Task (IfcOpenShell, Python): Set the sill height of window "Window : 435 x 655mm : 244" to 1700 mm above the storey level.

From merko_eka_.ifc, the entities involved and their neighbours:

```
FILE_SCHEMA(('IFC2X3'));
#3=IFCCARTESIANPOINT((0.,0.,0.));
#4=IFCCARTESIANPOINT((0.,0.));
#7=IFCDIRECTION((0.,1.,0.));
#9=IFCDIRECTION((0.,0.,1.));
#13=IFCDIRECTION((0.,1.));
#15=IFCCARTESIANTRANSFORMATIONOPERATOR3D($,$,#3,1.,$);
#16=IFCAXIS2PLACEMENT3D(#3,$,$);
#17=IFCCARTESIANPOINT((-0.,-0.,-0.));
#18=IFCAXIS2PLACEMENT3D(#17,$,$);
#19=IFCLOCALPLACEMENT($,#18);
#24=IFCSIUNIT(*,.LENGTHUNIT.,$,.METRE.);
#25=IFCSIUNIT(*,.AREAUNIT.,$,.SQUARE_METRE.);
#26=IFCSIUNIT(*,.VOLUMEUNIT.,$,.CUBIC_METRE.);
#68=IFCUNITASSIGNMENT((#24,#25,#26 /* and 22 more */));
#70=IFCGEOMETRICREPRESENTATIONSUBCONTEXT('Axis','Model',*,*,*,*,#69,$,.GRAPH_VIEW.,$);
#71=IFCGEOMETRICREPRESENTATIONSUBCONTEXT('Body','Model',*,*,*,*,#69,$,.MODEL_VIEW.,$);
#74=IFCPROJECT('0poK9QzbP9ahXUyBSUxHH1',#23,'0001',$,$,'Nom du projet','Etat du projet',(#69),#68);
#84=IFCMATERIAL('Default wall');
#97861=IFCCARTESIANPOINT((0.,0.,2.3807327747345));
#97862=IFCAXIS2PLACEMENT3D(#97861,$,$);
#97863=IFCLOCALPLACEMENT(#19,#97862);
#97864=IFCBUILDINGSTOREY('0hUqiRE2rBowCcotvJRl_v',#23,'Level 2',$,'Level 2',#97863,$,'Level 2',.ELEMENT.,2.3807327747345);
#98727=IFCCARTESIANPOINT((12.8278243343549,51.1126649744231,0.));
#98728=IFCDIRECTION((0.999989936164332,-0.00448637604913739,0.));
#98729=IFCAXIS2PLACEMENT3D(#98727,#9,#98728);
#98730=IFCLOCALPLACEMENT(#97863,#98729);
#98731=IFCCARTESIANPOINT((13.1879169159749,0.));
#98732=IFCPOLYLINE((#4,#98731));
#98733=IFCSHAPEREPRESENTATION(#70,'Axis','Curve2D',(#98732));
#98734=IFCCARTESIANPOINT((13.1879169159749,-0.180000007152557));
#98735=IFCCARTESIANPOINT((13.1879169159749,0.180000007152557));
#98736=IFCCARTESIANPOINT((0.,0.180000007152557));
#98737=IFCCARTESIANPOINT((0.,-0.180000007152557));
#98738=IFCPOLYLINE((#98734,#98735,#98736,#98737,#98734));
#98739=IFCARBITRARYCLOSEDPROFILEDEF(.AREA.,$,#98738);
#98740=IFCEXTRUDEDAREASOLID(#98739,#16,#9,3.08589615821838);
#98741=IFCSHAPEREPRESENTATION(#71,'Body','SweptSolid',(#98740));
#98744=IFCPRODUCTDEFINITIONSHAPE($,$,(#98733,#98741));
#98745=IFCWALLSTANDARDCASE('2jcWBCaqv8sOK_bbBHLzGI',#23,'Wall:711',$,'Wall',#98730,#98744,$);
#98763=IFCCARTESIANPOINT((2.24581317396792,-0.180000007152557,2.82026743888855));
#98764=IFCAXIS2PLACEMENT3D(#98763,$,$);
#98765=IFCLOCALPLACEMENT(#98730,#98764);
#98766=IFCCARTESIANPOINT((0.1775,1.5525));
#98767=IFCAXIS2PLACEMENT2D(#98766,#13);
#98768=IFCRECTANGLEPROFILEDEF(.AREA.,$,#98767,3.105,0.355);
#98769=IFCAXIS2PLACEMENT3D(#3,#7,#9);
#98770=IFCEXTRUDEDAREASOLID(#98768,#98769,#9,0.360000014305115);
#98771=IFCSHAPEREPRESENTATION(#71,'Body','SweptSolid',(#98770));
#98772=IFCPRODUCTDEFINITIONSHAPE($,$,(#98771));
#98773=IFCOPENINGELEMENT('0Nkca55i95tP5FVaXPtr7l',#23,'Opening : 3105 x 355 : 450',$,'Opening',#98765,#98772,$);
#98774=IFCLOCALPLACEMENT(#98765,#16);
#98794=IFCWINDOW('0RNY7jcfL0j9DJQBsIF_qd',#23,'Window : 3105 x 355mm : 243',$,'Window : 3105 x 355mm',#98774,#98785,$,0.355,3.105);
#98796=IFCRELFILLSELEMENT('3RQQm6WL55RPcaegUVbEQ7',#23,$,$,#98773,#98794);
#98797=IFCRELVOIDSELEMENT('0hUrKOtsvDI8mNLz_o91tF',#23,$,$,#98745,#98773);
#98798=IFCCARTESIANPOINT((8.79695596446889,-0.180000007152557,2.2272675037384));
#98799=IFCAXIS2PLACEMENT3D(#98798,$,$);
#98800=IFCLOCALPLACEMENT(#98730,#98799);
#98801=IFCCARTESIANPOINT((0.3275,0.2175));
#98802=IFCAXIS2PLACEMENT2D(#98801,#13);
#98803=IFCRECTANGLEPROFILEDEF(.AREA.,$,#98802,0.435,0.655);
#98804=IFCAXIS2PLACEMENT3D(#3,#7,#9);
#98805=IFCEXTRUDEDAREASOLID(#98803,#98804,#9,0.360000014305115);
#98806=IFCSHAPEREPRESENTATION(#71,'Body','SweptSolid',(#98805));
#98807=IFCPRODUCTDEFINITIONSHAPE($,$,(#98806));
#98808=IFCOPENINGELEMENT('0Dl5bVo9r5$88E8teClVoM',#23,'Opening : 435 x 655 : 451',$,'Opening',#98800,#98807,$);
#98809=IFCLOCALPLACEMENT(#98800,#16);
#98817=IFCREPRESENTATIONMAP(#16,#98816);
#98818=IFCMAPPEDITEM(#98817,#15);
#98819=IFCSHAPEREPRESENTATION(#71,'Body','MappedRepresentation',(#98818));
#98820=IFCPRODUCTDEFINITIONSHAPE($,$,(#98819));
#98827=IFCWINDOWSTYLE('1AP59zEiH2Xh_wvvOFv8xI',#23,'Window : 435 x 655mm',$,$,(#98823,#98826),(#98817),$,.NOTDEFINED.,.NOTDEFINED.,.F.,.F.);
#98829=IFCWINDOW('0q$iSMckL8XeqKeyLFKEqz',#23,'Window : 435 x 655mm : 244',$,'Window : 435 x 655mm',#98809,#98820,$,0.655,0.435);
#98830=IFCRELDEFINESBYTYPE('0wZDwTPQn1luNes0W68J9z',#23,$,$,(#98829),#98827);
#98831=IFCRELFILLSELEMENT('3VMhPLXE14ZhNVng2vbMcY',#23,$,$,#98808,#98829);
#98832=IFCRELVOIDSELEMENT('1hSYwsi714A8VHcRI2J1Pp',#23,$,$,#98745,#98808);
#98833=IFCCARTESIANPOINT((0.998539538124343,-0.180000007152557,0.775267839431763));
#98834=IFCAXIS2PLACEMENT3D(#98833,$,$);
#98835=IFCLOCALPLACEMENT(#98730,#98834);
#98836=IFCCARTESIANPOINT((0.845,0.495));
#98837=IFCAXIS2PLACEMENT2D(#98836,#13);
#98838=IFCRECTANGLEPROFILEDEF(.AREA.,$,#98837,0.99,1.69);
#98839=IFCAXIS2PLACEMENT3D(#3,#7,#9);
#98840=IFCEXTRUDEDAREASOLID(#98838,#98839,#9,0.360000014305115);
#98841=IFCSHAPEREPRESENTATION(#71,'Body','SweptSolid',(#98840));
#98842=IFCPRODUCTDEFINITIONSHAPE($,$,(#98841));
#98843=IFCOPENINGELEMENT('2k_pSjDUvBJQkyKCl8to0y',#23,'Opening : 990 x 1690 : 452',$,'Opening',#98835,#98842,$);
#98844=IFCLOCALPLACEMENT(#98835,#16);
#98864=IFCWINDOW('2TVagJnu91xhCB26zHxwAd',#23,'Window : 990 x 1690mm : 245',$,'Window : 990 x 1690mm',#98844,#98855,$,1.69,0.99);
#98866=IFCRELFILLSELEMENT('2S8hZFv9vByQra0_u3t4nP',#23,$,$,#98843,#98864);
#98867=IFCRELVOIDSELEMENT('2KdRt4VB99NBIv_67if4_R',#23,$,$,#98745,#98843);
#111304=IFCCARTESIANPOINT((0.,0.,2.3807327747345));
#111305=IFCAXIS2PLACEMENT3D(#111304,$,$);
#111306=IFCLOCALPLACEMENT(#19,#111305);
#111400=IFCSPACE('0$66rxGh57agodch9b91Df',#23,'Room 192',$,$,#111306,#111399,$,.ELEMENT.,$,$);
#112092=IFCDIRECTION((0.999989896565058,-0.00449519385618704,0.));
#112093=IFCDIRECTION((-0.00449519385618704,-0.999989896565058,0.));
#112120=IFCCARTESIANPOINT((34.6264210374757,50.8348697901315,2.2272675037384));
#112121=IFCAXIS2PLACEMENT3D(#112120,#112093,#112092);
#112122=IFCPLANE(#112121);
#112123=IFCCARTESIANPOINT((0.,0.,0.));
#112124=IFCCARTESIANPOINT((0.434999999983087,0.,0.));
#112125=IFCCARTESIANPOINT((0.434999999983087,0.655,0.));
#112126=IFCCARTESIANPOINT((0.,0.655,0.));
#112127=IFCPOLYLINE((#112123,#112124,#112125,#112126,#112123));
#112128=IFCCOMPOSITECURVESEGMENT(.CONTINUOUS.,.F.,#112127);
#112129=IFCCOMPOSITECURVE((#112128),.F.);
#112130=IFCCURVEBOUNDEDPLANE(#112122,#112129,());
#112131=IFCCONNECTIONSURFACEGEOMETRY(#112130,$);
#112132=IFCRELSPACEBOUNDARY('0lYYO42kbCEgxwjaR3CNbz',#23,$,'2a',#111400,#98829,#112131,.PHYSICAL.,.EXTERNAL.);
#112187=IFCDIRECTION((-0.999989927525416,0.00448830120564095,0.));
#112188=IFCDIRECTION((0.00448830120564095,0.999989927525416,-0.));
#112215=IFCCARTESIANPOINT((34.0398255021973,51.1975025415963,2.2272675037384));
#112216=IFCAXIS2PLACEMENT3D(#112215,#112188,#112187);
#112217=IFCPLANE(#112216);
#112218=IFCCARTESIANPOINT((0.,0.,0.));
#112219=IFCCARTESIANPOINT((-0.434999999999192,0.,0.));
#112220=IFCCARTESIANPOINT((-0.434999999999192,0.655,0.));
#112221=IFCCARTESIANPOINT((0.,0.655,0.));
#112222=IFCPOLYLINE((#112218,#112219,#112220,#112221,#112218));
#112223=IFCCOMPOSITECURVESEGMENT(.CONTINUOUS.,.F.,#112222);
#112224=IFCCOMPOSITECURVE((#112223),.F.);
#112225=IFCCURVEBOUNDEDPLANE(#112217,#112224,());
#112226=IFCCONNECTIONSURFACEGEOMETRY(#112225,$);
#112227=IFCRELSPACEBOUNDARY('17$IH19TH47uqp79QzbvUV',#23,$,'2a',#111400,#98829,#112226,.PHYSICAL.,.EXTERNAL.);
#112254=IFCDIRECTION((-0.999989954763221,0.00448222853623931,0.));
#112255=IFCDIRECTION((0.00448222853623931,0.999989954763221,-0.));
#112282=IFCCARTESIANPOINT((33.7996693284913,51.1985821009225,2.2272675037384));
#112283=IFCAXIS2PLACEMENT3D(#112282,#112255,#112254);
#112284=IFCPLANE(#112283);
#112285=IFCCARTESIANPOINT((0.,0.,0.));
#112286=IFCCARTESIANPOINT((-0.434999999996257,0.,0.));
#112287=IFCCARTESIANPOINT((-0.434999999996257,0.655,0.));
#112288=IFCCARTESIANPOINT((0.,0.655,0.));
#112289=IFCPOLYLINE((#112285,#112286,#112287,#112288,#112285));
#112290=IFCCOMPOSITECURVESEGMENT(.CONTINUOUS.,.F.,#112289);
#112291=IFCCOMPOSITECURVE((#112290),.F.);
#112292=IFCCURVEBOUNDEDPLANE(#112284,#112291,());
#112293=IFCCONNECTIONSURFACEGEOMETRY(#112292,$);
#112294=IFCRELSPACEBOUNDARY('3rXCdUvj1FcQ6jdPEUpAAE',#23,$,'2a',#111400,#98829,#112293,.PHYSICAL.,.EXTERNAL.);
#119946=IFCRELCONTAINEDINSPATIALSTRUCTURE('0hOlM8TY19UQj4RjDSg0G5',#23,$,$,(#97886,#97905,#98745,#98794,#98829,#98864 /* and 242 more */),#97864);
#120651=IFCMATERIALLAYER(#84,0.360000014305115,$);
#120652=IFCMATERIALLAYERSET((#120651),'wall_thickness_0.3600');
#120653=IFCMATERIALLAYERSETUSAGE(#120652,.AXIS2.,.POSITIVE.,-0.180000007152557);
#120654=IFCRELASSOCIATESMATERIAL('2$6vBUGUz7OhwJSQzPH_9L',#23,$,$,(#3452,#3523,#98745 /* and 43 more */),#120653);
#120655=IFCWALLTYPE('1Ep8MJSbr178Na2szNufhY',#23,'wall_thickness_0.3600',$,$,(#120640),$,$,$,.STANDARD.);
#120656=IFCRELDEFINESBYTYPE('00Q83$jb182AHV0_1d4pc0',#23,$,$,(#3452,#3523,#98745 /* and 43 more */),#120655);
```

```python
import numpy as np
import ifcopenshell
import ifcopenshell.api.geometry
import ifcopenshell.geom
import ifcopenshell.util.element
import ifcopenshell.util.placement
import ifcopenshell.util.shape
import ifcopenshell.util.unit

model = ifcopenshell.open("merko_eka_.ifc")
unit_scale = ifcopenshell.util.unit.calculate_unit_scale(model)

window = model.by_guid("0q$iSMckL8XeqKeyLFKEqz")
opening = window.FillsVoids[0].RelatingOpeningElement
storey = ifcopenshell.util.element.get_container(window, ifc_class="IfcBuildingStorey")
level = ifcopenshell.util.placement.get_local_placement(storey.ObjectPlacement)[2, 3]

# The opening's origin need not be at the sill, so measure its lowest point.
shape = ifcopenshell.geom.create_shape(ifcopenshell.geom.settings(), opening)
bottom = ifcopenshell.util.shape.get_shape_bottom_elevation(shape, shape.geometry) / unit_scale
dz = level + 1.7 / unit_scale - bottom

shift = np.array([0.0, 0.0, dz])
# The window is placed relative to its opening, so it follows when the opening moves.
matrix = ifcopenshell.util.placement.get_local_placement(opening.ObjectPlacement)
matrix[:3, 3] += shift
ifcopenshell.api.geometry.edit_object_placement(
    model, product=opening, matrix=matrix, is_si=False, should_transform_children=True
)

# Space boundary surfaces are stored in each space's coordinates; move them too.
for rel in window.ProvidesBoundaries:
    if not rel.ConnectionGeometry:
        continue
    surface = rel.ConnectionGeometry.SurfaceOnRelatingElement.BasisSurface
    space_matrix = ifcopenshell.util.placement.get_local_placement(rel.RelatingSpace.ObjectPlacement)
    point = np.array(surface.Position.Location.Coordinates) + space_matrix[:3, :3].T @ shift
    surface.Position = model.createIfcAxis2Placement3D(
        model.createIfcCartesianPoint(point.tolist()), surface.Position.Axis, surface.Position.RefDirection
    )

print(f"moved by {dz * unit_scale:+.3f} m")

model.write("merko_eka__edited.ifc")
```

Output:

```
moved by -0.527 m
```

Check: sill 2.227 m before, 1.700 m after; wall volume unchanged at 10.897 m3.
